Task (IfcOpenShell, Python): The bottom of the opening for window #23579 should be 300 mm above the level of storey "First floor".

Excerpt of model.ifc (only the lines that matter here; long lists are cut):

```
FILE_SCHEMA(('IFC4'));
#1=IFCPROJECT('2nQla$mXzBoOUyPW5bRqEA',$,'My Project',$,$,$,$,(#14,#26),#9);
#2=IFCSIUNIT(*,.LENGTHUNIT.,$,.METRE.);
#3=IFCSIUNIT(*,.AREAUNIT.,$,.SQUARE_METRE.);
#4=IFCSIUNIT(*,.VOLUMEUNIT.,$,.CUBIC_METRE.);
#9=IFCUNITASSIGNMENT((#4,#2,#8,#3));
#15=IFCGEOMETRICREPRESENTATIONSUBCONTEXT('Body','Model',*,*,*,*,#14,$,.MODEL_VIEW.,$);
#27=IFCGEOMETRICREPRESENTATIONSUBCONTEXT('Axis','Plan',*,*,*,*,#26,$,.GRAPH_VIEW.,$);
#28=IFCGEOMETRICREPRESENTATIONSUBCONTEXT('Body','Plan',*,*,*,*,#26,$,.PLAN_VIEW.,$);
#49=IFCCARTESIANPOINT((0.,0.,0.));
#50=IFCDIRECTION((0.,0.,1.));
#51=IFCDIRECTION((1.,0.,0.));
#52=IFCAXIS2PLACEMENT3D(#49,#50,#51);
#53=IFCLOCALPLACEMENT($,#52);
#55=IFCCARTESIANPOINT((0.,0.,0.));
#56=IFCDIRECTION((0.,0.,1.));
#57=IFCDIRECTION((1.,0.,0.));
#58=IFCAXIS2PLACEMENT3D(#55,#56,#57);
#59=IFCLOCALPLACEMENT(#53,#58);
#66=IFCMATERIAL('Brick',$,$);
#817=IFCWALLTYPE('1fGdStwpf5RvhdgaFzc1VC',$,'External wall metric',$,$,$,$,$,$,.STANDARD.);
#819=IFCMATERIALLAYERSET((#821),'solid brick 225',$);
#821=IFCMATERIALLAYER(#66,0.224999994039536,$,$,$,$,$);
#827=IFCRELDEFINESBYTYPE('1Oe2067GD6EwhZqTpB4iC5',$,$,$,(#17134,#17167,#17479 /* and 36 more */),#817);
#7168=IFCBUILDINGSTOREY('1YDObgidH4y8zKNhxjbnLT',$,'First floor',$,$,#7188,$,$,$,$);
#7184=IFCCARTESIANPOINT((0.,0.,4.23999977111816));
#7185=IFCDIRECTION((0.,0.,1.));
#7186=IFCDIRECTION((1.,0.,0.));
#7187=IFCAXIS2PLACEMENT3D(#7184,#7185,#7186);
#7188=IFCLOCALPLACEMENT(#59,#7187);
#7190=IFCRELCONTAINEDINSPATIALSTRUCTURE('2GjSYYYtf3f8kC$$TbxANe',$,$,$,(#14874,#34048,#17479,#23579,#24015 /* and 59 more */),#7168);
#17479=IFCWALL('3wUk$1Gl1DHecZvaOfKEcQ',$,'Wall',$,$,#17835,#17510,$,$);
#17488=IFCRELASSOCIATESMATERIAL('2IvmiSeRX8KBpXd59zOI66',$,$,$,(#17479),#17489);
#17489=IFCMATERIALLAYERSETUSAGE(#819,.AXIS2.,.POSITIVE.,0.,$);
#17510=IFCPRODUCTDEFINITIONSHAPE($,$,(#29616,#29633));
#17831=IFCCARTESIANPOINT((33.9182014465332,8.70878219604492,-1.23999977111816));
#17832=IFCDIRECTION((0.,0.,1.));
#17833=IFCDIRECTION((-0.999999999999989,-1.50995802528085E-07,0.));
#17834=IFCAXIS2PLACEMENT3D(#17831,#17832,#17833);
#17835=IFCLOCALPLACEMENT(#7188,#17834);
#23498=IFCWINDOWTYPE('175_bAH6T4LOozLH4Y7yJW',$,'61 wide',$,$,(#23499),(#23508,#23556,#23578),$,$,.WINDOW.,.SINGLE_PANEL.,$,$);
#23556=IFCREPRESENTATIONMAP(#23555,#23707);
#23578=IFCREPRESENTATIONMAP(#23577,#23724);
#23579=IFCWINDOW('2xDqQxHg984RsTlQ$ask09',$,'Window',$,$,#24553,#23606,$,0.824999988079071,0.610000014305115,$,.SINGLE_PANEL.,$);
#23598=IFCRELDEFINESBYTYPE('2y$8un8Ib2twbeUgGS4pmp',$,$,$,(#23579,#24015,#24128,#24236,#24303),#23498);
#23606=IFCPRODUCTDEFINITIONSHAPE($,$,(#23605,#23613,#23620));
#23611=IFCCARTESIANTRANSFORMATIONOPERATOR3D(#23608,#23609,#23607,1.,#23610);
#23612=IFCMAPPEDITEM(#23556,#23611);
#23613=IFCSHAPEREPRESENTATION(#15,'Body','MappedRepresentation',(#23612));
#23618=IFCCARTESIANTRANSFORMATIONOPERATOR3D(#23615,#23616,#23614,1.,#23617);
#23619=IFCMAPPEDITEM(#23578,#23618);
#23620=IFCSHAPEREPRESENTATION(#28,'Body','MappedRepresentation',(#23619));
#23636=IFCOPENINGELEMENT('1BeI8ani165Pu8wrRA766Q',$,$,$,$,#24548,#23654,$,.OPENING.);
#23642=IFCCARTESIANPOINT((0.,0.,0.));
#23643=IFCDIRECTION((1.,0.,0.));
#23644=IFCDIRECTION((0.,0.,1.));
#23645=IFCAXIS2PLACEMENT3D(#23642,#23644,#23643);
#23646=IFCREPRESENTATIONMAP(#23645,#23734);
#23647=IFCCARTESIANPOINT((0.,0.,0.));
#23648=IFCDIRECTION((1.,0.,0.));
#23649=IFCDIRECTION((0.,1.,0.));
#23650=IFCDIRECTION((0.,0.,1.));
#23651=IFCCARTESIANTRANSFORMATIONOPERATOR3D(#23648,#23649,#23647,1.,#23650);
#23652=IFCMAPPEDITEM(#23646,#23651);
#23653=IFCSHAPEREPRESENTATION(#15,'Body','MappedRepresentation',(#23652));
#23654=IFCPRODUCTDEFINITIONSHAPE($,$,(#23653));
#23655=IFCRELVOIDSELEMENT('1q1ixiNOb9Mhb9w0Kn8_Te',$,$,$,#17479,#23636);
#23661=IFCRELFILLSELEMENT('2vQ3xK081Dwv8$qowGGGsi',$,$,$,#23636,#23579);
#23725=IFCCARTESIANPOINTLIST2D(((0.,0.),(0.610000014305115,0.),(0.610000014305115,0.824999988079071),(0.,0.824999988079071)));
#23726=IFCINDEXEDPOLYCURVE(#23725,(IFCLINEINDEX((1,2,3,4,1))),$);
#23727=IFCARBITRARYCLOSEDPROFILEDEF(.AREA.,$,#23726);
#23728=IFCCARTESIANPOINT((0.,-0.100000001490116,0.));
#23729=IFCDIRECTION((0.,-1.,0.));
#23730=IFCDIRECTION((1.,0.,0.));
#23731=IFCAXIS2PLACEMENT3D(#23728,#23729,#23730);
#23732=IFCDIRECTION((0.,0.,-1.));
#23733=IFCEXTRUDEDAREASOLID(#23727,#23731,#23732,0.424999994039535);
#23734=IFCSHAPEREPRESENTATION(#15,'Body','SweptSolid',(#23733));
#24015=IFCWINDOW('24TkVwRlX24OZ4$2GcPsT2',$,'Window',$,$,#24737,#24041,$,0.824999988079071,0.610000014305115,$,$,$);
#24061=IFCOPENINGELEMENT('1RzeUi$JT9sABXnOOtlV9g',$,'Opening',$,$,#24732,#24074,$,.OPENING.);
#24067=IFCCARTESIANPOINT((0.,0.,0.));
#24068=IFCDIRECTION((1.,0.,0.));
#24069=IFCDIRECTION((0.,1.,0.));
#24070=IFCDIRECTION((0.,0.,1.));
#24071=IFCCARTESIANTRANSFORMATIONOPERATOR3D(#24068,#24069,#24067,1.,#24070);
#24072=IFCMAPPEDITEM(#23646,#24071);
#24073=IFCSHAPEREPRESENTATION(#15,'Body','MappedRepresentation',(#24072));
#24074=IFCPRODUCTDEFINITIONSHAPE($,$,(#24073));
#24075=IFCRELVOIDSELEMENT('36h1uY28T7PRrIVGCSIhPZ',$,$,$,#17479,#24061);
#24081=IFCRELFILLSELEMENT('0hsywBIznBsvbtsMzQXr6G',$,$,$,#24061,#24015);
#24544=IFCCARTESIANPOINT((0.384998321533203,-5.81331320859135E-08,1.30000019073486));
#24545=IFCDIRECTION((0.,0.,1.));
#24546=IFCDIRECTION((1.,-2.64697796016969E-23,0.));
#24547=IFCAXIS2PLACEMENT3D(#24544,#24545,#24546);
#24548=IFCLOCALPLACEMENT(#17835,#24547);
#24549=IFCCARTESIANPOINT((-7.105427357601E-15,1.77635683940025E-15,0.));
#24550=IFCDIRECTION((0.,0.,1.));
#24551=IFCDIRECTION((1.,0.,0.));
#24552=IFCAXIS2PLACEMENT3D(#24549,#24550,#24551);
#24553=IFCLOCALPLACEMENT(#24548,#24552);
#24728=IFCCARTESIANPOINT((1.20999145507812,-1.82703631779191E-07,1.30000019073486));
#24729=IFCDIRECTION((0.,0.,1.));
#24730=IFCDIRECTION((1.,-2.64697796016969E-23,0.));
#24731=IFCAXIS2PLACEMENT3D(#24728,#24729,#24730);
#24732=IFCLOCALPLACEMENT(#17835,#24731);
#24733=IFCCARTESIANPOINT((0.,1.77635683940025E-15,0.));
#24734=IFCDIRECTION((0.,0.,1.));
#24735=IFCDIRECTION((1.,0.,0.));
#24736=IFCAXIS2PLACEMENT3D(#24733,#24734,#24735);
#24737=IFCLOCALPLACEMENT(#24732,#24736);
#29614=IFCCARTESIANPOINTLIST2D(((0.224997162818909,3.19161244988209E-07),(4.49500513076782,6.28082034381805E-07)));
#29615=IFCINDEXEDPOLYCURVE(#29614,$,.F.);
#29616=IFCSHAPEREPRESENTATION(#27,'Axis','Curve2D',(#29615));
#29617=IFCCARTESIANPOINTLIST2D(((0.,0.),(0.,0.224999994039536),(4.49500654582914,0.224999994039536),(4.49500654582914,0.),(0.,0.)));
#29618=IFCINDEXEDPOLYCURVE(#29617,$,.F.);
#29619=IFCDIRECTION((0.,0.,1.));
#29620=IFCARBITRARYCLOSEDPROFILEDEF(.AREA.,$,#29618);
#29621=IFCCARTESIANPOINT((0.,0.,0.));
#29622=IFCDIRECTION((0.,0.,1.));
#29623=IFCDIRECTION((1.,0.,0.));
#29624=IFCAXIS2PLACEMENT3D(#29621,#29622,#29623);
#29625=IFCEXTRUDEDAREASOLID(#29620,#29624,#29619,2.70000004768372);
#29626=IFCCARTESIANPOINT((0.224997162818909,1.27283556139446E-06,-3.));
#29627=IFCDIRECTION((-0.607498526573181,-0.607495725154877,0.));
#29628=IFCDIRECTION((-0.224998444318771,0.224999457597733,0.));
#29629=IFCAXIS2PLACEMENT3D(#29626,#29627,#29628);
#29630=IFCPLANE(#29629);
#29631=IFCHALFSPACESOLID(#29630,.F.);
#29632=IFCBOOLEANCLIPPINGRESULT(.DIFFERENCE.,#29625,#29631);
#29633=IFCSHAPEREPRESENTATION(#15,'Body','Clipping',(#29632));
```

```python
import numpy as np
import ifcopenshell
import ifcopenshell.api.geometry
import ifcopenshell.geom
import ifcopenshell.util.element
import ifcopenshell.util.placement
import ifcopenshell.util.shape
import ifcopenshell.util.unit

model = ifcopenshell.open("model.ifc")
unit_scale = ifcopenshell.util.unit.calculate_unit_scale(model)

window = model.by_guid("2xDqQxHg984RsTlQ$ask09")
opening = window.FillsVoids[0].RelatingOpeningElement
storey = ifcopenshell.util.element.get_container(window, ifc_class="IfcBuildingStorey")
level = ifcopenshell.util.placement.get_local_placement(storey.ObjectPlacement)[2, 3]

# The opening's origin need not be at the sill, so measure its lowest point.
shape = ifcopenshell.geom.create_shape(ifcopenshell.geom.settings(), opening)
bottom = ifcopenshell.util.shape.get_shape_bottom_elevation(shape, shape.geometry) / unit_scale
dz = level + 0.3 / unit_scale - bottom

shift = np.array([0.0, 0.0, dz])
# The window is placed relative to its opening, so it follows when the opening moves.
matrix = ifcopenshell.util.placement.get_local_placement(opening.ObjectPlacement)
matrix[:3, 3] += shift
ifcopenshell.api.geometry.edit_object_placement(
    model, product=opening, matrix=matrix, is_si=False, should_transform_children=True
)

print(f"moved by {dz * unit_scale:+.3f} m")

model.write("model_rev.ifc")
```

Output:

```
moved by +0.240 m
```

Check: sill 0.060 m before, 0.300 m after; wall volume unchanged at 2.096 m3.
